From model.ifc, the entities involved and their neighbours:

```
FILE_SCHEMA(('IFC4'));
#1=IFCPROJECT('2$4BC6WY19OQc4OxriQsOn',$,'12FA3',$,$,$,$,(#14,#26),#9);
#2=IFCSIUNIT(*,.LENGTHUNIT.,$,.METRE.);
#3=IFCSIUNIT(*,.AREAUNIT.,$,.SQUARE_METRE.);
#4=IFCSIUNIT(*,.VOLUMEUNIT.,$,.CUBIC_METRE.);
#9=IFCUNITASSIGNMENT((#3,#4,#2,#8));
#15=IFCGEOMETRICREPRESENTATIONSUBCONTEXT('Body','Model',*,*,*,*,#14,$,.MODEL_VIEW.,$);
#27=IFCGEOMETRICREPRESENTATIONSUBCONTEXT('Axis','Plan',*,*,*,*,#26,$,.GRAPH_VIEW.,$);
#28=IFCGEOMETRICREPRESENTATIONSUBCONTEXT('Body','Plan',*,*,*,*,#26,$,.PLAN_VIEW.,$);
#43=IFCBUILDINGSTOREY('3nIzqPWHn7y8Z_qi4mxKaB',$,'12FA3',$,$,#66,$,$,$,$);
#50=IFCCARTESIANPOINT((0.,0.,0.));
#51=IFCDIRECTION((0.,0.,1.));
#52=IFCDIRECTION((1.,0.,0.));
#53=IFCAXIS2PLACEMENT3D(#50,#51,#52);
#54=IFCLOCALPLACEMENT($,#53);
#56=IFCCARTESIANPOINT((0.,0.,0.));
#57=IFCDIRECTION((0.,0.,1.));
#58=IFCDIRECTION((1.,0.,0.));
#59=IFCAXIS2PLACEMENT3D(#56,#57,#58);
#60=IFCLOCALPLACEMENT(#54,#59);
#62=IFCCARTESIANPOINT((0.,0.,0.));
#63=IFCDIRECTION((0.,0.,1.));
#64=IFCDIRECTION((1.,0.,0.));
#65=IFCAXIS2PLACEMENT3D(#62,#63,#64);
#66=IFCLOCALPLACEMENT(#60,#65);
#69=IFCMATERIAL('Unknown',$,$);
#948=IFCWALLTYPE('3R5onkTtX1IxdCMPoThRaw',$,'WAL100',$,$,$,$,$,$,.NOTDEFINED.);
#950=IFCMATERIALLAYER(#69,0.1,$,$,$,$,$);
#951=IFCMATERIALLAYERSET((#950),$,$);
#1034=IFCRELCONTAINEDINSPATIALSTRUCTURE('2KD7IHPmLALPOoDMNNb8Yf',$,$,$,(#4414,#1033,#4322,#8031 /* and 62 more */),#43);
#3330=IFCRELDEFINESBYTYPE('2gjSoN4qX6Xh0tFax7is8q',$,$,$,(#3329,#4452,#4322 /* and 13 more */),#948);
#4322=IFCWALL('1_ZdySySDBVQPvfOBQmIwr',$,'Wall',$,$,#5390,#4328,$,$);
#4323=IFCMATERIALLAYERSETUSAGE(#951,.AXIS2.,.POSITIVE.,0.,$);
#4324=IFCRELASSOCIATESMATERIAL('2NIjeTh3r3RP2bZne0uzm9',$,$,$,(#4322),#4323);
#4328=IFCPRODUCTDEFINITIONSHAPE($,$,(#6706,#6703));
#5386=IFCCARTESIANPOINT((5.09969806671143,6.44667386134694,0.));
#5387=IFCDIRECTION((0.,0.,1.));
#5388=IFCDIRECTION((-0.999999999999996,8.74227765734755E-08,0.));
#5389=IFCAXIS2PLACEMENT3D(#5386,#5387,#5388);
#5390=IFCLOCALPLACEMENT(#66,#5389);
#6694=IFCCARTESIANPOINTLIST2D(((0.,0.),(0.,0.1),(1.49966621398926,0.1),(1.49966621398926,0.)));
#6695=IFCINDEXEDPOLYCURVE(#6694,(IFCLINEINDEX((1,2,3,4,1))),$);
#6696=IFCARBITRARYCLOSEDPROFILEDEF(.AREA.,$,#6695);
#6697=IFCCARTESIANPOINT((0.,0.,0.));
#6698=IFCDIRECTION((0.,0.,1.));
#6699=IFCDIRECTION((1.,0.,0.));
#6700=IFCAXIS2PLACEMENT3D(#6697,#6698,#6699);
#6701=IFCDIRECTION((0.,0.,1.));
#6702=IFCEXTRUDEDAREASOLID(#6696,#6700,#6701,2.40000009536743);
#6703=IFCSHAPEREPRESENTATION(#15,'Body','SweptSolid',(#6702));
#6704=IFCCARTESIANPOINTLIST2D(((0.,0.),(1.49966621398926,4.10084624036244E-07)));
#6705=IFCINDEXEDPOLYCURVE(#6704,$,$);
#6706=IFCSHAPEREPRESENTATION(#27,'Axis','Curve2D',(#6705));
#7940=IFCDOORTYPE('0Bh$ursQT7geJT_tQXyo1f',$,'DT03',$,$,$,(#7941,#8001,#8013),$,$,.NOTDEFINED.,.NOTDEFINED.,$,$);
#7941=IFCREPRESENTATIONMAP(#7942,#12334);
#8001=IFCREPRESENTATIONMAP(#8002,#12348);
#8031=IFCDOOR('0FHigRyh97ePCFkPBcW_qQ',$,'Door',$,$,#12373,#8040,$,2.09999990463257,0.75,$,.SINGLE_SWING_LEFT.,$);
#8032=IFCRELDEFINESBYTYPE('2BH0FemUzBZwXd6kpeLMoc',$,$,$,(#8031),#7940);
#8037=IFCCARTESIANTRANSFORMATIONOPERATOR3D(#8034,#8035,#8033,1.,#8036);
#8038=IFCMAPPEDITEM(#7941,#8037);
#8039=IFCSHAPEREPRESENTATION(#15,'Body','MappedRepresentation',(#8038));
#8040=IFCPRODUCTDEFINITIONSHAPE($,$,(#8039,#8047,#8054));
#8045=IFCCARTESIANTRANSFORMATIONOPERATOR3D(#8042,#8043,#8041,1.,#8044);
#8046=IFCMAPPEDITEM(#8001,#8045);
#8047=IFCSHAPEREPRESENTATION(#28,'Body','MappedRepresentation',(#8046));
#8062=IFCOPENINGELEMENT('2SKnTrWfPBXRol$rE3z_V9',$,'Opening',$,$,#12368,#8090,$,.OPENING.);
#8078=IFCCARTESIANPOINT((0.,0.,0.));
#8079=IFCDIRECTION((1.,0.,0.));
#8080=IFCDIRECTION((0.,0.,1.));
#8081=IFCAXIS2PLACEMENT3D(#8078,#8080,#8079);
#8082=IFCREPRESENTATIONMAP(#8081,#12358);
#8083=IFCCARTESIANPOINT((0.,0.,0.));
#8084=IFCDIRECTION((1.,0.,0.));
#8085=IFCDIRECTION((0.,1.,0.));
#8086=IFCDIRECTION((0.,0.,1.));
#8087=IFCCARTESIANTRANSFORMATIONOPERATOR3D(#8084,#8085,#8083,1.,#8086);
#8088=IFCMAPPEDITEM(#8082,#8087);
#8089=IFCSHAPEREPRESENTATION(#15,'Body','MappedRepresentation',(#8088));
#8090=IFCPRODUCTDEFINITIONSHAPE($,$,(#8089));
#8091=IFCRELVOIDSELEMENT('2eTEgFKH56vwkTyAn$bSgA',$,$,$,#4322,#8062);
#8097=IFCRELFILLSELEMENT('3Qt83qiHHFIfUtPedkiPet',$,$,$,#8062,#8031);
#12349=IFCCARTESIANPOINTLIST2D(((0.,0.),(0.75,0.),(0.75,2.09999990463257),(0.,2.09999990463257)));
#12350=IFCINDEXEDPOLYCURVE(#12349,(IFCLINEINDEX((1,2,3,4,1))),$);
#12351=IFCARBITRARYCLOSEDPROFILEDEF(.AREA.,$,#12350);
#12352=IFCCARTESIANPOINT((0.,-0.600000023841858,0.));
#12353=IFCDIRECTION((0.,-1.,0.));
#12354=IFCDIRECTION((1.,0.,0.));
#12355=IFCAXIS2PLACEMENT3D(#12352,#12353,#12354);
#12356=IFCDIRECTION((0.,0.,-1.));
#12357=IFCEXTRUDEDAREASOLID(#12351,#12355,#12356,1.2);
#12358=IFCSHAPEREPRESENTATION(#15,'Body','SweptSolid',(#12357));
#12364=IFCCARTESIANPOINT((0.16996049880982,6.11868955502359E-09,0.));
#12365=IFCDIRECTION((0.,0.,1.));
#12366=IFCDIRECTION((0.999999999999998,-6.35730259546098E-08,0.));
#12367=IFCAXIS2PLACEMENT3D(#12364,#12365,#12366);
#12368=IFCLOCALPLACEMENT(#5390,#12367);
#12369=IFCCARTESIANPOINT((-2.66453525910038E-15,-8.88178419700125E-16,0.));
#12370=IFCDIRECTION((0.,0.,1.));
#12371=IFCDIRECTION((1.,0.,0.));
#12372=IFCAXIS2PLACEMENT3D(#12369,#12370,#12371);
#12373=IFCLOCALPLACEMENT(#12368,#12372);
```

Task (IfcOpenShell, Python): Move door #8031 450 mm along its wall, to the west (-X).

```python
import ifcopenshell
import ifcopenshell.api.geometry
import ifcopenshell.util.placement
import ifcopenshell.util.unit

model = ifcopenshell.open("model.ifc")
unit_scale = ifcopenshell.util.unit.calculate_unit_scale(model)

door = model.by_guid("0FHigRyh97ePCFkPBcW_qQ")
opening = door.FillsVoids[0].RelatingOpeningElement
wall = opening.VoidsElements[0].RelatingBuildingElement

wall_matrix = ifcopenshell.util.placement.get_local_placement(wall.ObjectPlacement)
shift = wall_matrix[:3, 0] * 0.45 / unit_scale
before = ifcopenshell.util.placement.get_local_placement(door.ObjectPlacement)[:3, 3].copy()

# The door is placed relative to its opening, so it follows when the opening moves.
matrix = ifcopenshell.util.placement.get_local_placement(opening.ObjectPlacement)
matrix[:3, 3] += shift
ifcopenshell.api.geometry.edit_object_placement(
    model, product=opening, matrix=matrix, is_si=False, should_transform_children=True
)

after = ifcopenshell.util.placement.get_local_placement(door.ObjectPlacement)[:3, 3]
print("door moved by", (after - before).round(3) + 0.0)

model.write("model_edited.ifc")
```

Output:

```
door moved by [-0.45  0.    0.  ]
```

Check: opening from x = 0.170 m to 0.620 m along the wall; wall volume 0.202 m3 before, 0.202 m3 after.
